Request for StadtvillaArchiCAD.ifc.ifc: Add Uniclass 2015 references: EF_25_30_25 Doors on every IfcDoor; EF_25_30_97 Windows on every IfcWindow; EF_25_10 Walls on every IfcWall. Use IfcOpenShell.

First a look at what the model holds.

```python
import ifcopenshell

model = ifcopenshell.open("StadtvillaArchiCAD.ifc.ifc")
print(model.schema)
print("classifications:", [c.Name for c in model.by_type("IfcClassification")])
for ifc_class in ("IfcDoor", "IfcRoof", "IfcStair", "IfcWall", "IfcWindow"):
    print(ifc_class, len(model.by_type(ifc_class)))
```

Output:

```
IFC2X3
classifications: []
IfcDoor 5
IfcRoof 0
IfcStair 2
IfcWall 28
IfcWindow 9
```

```python
import ifcopenshell
import ifcopenshell.api.classification

model = ifcopenshell.open("StadtvillaArchiCAD.ifc.ifc")

# IFC2X3 requires Source and Edition and has no link from the project to the system.
system = model.create_entity("IfcClassification", Source="NBS", Edition="2015", Name="Uniclass 2015")

codes = {
    "IfcDoor": ("EF_25_30_25", "Doors"),
    "IfcWindow": ("EF_25_30_97", "Windows"),
    "IfcWall": ("EF_25_10", "Walls"),
}
for ifc_class, (code, name) in codes.items():
    products = model.by_type(ifc_class)
    ifcopenshell.api.classification.add_reference(
        model, products=products, classification=system, identification=code, name=name
    )
    print(code, len(products))

model.write("StadtvillaArchiCAD.ifc_updated.ifc")
```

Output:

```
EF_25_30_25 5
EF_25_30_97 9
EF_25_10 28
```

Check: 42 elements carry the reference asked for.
